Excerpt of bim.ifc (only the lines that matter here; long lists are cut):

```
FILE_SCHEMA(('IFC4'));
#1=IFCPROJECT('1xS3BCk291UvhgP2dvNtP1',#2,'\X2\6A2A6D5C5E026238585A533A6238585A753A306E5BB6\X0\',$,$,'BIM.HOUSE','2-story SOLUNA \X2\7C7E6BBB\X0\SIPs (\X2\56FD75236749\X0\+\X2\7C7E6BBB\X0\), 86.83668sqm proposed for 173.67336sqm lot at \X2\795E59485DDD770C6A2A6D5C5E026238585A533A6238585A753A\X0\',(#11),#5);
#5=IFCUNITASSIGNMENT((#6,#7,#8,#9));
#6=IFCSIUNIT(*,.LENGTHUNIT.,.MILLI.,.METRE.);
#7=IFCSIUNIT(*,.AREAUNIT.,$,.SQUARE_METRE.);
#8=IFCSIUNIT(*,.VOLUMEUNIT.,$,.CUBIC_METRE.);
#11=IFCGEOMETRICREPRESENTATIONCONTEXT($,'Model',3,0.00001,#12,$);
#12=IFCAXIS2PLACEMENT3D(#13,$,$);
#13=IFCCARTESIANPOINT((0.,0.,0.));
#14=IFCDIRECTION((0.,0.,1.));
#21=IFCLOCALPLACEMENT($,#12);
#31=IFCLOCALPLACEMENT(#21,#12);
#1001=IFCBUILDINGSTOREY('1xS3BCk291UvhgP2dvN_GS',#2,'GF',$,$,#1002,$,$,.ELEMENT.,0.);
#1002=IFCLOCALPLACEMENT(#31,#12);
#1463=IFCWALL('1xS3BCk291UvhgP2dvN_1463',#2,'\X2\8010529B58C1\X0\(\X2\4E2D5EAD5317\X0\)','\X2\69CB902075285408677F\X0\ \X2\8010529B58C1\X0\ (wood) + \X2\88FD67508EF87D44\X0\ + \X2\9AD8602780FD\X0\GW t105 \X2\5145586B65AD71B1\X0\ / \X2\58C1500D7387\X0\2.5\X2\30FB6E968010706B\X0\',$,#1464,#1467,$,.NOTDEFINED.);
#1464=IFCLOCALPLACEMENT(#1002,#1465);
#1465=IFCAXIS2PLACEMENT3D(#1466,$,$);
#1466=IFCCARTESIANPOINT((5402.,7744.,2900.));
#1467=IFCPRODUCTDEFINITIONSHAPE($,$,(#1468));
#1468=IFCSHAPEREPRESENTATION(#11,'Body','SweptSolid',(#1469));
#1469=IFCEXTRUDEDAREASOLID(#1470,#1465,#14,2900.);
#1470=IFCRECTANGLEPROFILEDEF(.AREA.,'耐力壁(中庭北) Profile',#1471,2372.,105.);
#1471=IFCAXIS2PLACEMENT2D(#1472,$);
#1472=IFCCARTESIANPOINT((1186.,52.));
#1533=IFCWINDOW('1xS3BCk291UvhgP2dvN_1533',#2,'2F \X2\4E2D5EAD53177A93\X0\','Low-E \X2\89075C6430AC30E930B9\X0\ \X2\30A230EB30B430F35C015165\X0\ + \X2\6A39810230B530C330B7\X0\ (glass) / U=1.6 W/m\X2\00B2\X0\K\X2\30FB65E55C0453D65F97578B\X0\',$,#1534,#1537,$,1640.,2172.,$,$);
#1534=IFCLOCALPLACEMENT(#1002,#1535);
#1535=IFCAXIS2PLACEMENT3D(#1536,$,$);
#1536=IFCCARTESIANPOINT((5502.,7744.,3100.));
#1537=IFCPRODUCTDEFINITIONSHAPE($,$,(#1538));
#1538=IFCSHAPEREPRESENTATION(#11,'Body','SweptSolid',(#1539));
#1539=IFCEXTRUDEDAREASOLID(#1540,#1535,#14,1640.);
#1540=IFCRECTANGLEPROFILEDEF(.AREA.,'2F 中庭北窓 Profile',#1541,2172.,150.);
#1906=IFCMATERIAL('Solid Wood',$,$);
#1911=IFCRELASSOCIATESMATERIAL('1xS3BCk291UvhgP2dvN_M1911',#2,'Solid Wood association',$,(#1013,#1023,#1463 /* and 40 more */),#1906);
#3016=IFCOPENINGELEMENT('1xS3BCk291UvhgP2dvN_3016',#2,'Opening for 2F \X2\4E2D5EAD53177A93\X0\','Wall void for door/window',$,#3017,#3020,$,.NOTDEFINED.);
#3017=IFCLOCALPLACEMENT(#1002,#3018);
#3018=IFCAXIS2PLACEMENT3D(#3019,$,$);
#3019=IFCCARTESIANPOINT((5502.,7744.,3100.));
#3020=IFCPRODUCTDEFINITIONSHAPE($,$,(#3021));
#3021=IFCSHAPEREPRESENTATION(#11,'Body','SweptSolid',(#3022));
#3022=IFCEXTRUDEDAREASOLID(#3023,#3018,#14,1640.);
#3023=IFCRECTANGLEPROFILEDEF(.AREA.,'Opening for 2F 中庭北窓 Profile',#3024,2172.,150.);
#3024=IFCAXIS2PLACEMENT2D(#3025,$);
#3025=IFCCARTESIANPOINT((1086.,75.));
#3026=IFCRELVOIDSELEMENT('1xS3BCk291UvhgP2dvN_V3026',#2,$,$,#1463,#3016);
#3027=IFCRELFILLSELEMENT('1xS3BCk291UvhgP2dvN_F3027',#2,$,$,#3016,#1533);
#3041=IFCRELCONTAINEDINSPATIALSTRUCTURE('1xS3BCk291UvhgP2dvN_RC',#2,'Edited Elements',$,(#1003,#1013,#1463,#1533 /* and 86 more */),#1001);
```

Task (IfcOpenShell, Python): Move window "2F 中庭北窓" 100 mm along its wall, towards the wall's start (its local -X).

```python
import ifcopenshell
import ifcopenshell.api.geometry
import ifcopenshell.util.placement
import ifcopenshell.util.unit

model = ifcopenshell.open("bim.ifc")
unit_scale = ifcopenshell.util.unit.calculate_unit_scale(model)

window = model.by_guid("1xS3BCk291UvhgP2dvN_1533")
opening = window.FillsVoids[0].RelatingOpeningElement
wall = opening.VoidsElements[0].RelatingBuildingElement

wall_matrix = ifcopenshell.util.placement.get_local_placement(wall.ObjectPlacement)
shift = wall_matrix[:3, 0] * -0.1 / unit_scale
before = ifcopenshell.util.placement.get_local_placement(window.ObjectPlacement)[:3, 3].copy()

# The window is not placed relative to its opening, so move both.
for product in (opening, window):
    matrix = ifcopenshell.util.placement.get_local_placement(product.ObjectPlacement)
    matrix[:3, 3] += shift
    ifcopenshell.api.geometry.edit_object_placement(model, product=product, matrix=matrix, is_si=False)

after = ifcopenshell.util.placement.get_local_placement(window.ObjectPlacement)[:3, 3]
print("window moved by", (after - before).round(3) + 0.0)

model.write("bim_rev.ifc")
```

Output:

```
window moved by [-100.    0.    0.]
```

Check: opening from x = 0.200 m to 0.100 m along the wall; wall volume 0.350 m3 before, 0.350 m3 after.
